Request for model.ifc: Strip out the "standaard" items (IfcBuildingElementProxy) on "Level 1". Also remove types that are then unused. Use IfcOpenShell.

First a look at what the model holds.

```python
import ifcopenshell
import ifcopenshell.util.element

model = ifcopenshell.open("model.ifc")
print(model.schema)
storey = next(s for s in model.by_type("IfcBuildingStorey") if s.Name == "Level 1")
proxies = [e for e in ifcopenshell.util.element.get_decomposition(storey) if e.is_a("IfcBuildingElementProxy")]
seen = {}
for e in proxies:
    element_type = ifcopenshell.util.element.get_type(e)
    name = element_type.Name if element_type not in (None, e) else None
    seen[name] = seen.get(name, 0) + 1
for name, count in sorted(seen.items(), key=str):
    print(count, "x", name)
```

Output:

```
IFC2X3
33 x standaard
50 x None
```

```python
import ifcopenshell
import ifcopenshell.api.root
import ifcopenshell.util.element

model = ifcopenshell.open("model.ifc")

storey = next(s for s in model.by_type("IfcBuildingStorey") if s.Name == "Level 1")
proxies = [e for e in ifcopenshell.util.element.get_decomposition(storey) if e.is_a("IfcBuildingElementProxy")]
targets = [e for e in proxies if (t := ifcopenshell.util.element.get_type(e)) not in (None, e) and t.Name == "standaard"]
types = {ifcopenshell.util.element.get_type(e) for e in targets} - {None, *targets}

for e in targets:
    ifcopenshell.api.root.remove_product(model, product=e)
print(len(targets), "removed")

unused = [t for t in types if not ifcopenshell.util.element.get_types(t)]
for t in unused:
    ifcopenshell.api.root.remove_product(model, product=t)
print(len(unused), "unused types removed")

model.write("model_updated.ifc")
```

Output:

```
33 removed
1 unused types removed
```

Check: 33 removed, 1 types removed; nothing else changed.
